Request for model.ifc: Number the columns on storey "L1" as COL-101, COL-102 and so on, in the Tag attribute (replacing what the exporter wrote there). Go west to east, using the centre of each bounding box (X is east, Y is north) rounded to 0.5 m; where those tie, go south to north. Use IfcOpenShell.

First a look at what the model holds.

```python
import ifcopenshell
import ifcopenshell.util.element
import ifcopenshell.util.placement

model = ifcopenshell.open("model.ifc")
print(model.schema)
storey = next(s for s in model.by_type("IfcBuildingStorey") if s.Name == "L1")
columns = [e for e in ifcopenshell.util.element.get_decomposition(storey) if e.is_a("IfcColumn")]
for e in sorted(columns, key=lambda e: e.id()):
    origin = ifcopenshell.util.placement.get_local_placement(e.ObjectPlacement)[:3, 3]
    print(e.id(), e.Tag, e.Name, origin.round(2) + 0.0, sep=" | ")
```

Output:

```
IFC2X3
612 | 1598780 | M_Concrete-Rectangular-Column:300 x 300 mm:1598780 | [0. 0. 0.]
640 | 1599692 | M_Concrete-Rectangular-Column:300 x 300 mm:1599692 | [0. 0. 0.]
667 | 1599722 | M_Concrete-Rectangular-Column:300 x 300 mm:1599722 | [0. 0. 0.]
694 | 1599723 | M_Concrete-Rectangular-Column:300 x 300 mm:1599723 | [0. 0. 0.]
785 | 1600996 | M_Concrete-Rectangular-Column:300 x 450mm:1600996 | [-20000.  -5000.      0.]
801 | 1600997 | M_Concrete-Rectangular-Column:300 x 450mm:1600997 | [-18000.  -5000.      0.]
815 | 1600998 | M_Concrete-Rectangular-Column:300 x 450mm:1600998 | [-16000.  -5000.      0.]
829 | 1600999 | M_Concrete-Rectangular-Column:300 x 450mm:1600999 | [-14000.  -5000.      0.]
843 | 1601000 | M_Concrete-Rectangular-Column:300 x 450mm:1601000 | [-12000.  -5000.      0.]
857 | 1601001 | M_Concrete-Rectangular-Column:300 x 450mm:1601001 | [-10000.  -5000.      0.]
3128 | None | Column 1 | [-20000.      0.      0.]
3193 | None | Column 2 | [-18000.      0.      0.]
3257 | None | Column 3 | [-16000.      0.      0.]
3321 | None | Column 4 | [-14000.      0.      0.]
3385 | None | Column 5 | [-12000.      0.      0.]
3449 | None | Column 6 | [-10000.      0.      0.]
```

```python
import ifcopenshell
import ifcopenshell.geom
import ifcopenshell.util.element
import ifcopenshell.util.shape

model = ifcopenshell.open("model.ifc")
settings = ifcopenshell.geom.settings()
settings.set("use-world-coords", True)


def centre(element):
    shape = ifcopenshell.geom.create_shape(settings, element)
    return ifcopenshell.util.shape.get_bbox_centroid(shape.geometry)


storey = next(s for s in model.by_type("IfcBuildingStorey") if s.Name == "L1")
columns = [e for e in ifcopenshell.util.element.get_decomposition(storey) if e.is_a("IfcColumn")]

# Insertion points can sit at a corner or the storey origin, so sort by the geometry (in metres).
centres = {e: centre(e) for e in columns}
columns.sort(key=lambda e: (round(centres[e][0] / 0.5), centres[e][1]))

for i, e in enumerate(columns, start=1):
    number = f"COL-1{i:02d}"
    e.Tag = number
    print(e.id(), number)

model.write("model_rev.ifc")
```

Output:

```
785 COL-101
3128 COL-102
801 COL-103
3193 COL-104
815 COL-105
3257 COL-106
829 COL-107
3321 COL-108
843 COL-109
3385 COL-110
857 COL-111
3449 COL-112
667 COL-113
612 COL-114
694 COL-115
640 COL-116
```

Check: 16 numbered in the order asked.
